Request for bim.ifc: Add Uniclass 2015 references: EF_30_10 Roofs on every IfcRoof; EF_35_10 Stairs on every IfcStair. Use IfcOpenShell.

First a look at what the model holds.

```python
import ifcopenshell

model = ifcopenshell.open("bim.ifc")
print(model.schema)
print("classifications:", [c.Name for c in model.by_type("IfcClassification")])
for ifc_class in ("IfcDoor", "IfcRoof", "IfcStair", "IfcWall", "IfcWindow"):
    print(ifc_class, len(model.by_type(ifc_class)))
```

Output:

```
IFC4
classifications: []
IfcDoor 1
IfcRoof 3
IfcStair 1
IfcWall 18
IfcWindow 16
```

```python
import ifcopenshell
import ifcopenshell.api.classification

model = ifcopenshell.open("bim.ifc")

system = ifcopenshell.api.classification.add_classification(model, classification="Uniclass 2015")

codes = {
    "IfcRoof": ("EF_30_10", "Roofs"),
    "IfcStair": ("EF_35_10", "Stairs"),
}
for ifc_class, (code, name) in codes.items():
    products = model.by_type(ifc_class)
    ifcopenshell.api.classification.add_reference(
        model, products=products, classification=system, identification=code, name=name
    )
    print(code, len(products))

model.write("bim-out.ifc")
```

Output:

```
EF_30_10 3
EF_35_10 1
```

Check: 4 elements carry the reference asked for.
